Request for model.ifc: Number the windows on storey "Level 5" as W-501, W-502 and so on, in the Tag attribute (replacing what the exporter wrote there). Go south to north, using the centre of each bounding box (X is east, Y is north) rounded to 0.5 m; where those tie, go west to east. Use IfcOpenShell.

First a look at what the model holds.

```python
import ifcopenshell
import ifcopenshell.util.element
import ifcopenshell.util.placement

model = ifcopenshell.open("model.ifc")
print(model.schema)
storey = next(s for s in model.by_type("IfcBuildingStorey") if s.Name == "Level 5")
windows = [e for e in ifcopenshell.util.element.get_decomposition(storey) if e.is_a("IfcWindow")]
for e in sorted(windows, key=lambda e: e.id()):
    origin = ifcopenshell.util.placement.get_local_placement(e.ObjectPlacement)[:3, 3]
    print(e.id(), e.Tag, e.Name, origin.round(2) + 0.0, sep=" | ")
```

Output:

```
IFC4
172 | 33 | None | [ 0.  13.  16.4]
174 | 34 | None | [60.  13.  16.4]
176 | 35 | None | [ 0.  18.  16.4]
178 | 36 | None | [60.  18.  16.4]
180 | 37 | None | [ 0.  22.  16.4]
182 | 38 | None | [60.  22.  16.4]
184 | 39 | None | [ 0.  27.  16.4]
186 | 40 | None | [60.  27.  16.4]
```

```python
import ifcopenshell
import ifcopenshell.geom
import ifcopenshell.util.element
import ifcopenshell.util.shape

model = ifcopenshell.open("model.ifc")
settings = ifcopenshell.geom.settings()
settings.set("use-world-coords", True)


def centre(element):
    shape = ifcopenshell.geom.create_shape(settings, element)
    return ifcopenshell.util.shape.get_bbox_centroid(shape.geometry)


storey = next(s for s in model.by_type("IfcBuildingStorey") if s.Name == "Level 5")
windows = [e for e in ifcopenshell.util.element.get_decomposition(storey) if e.is_a("IfcWindow")]

# Insertion points can sit at a corner or the storey origin, so sort by the geometry (in metres).
centres = {e: centre(e) for e in windows}
windows.sort(key=lambda e: (round(centres[e][1] / 0.5), centres[e][0]))

for i, e in enumerate(windows, start=1):
    number = f"W-5{i:02d}"
    e.Tag = number
    print(e.id(), number)

model.write("model_edited.ifc")
```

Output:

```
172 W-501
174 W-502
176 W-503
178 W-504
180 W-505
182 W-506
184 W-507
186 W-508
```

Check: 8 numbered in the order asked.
